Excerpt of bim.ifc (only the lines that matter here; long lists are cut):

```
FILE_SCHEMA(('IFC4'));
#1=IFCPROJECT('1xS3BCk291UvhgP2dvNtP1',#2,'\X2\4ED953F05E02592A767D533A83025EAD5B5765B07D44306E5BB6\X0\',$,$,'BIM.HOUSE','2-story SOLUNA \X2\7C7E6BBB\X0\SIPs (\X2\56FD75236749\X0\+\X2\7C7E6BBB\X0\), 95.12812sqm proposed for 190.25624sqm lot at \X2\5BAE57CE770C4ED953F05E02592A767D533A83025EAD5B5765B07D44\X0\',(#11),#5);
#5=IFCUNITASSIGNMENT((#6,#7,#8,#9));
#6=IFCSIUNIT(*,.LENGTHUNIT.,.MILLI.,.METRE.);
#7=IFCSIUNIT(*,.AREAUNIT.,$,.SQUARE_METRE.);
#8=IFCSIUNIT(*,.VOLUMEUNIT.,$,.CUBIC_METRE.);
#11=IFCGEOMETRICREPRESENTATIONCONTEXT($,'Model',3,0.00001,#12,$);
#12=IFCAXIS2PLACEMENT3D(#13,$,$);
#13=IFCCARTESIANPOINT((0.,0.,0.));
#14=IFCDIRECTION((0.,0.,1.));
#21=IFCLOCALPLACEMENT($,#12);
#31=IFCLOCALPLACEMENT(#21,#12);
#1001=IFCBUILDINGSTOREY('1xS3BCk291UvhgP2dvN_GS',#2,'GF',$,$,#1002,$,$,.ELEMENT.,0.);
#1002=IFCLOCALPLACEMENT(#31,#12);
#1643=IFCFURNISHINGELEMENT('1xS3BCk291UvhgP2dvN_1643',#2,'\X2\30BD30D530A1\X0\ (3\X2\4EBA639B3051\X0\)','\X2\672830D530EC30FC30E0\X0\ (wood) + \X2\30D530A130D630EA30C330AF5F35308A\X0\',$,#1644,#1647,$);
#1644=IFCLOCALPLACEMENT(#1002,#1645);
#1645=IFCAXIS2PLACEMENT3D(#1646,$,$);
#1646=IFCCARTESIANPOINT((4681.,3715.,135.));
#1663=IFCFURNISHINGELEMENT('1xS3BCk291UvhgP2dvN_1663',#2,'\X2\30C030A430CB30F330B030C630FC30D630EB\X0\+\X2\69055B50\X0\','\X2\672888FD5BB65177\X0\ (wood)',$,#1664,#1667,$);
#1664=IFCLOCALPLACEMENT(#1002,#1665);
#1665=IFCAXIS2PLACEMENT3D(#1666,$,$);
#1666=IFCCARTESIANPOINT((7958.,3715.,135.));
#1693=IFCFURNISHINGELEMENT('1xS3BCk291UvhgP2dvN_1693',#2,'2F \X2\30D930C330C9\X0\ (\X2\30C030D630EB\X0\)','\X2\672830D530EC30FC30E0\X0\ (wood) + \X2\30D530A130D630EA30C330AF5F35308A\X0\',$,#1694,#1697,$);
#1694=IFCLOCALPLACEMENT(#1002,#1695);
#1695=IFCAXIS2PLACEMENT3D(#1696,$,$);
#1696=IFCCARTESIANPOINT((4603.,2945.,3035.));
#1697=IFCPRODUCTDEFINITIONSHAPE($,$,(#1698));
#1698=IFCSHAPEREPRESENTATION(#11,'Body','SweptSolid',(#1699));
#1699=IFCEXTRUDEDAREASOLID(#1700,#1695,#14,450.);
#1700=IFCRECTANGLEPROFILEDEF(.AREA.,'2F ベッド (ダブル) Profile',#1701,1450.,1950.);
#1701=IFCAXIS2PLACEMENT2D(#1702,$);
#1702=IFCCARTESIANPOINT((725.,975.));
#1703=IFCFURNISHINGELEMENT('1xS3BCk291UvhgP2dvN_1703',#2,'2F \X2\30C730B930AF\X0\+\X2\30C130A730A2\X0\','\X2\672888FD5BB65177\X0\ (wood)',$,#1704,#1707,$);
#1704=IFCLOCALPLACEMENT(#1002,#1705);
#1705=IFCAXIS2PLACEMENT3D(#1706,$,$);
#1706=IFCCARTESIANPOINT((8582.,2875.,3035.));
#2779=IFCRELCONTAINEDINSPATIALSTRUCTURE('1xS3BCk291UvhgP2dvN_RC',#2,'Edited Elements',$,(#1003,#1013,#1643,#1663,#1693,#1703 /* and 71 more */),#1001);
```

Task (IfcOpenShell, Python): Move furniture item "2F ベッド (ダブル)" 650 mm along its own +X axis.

```python
import ifcopenshell
import ifcopenshell.api.geometry
import ifcopenshell.util.placement
import ifcopenshell.util.unit

model = ifcopenshell.open("bim.ifc")
unit_scale = ifcopenshell.util.unit.calculate_unit_scale(model)

item = model.by_guid("1xS3BCk291UvhgP2dvN_1693")
matrix = ifcopenshell.util.placement.get_local_placement(item.ObjectPlacement)
matrix[:3, 3] += matrix[:3, 0] * 0.65 / unit_scale
ifcopenshell.api.geometry.edit_object_placement(model, product=item, matrix=matrix, is_si=False)

print(ifcopenshell.util.placement.get_local_placement(item.ObjectPlacement).round(3) + 0.0)

model.write("bim_edited.ifc")
```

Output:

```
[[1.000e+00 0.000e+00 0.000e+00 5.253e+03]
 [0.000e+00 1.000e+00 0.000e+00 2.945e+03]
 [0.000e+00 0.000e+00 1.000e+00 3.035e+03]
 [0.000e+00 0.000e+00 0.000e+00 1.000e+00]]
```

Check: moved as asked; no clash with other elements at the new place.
